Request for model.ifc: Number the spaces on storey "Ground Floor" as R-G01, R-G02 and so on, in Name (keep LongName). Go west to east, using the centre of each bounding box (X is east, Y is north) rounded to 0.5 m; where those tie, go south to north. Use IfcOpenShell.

First a look at what the model holds.

```python
import ifcopenshell
import ifcopenshell.util.element
import ifcopenshell.util.placement

model = ifcopenshell.open("model.ifc")
print(model.schema)
storey = next(s for s in model.by_type("IfcBuildingStorey") if s.Name == "Ground Floor")
spaces = [e for e in ifcopenshell.util.element.get_decomposition(storey) if e.is_a("IfcSpace")]
for e in sorted(spaces, key=lambda e: e.id()):
    origin = ifcopenshell.util.placement.get_local_placement(e.ObjectPlacement)[:3, 3]
    print(e.id(), e.Name, e.LongName, origin.round(2) + 0.0, sep=" | ")
```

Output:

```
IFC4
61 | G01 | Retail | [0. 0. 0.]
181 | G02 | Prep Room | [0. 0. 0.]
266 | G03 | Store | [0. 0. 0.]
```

```python
import ifcopenshell
import ifcopenshell.geom
import ifcopenshell.util.element
import ifcopenshell.util.shape

model = ifcopenshell.open("model.ifc")
settings = ifcopenshell.geom.settings()
settings.set("use-world-coords", True)


def centre(element):
    shape = ifcopenshell.geom.create_shape(settings, element)
    return ifcopenshell.util.shape.get_bbox_centroid(shape.geometry)


storey = next(s for s in model.by_type("IfcBuildingStorey") if s.Name == "Ground Floor")
spaces = [e for e in ifcopenshell.util.element.get_decomposition(storey) if e.is_a("IfcSpace")]

# Insertion points can sit at a corner or the storey origin, so sort by the geometry (in metres).
centres = {e: centre(e) for e in spaces}
spaces.sort(key=lambda e: (round(centres[e][0] / 0.5), centres[e][1]))

for i, e in enumerate(spaces, start=1):
    number = f"R-G{i:02d}"
    e.Name = number
    print(e.id(), number)

model.write("model_rev.ifc")
```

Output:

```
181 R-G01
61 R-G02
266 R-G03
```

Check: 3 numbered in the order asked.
